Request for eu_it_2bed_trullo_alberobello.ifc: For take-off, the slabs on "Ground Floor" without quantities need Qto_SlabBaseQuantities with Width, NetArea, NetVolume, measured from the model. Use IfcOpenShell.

First a look at what the model holds.

```python
import ifcopenshell
import ifcopenshell.util.element
import ifcopenshell.util.unit

model = ifcopenshell.open("eu_it_2bed_trullo_alberobello.ifc")
print(model.schema)
for unit_type in ("LENGTHUNIT", "AREAUNIT", "VOLUMEUNIT"):
    print(unit_type, ifcopenshell.util.unit.calculate_unit_scale(model, unit_type))
storey = next(s for s in model.by_type("IfcBuildingStorey") if s.Name == "Ground Floor")
slabs = [e for e in ifcopenshell.util.element.get_decomposition(storey) if e.is_a("IfcSlab")]
for e in sorted(slabs, key=lambda e: e.id()):
    print(e.id(), e.is_a(), e.Name, list(ifcopenshell.util.element.get_psets(e, qtos_only=True)), sep=" | ")
```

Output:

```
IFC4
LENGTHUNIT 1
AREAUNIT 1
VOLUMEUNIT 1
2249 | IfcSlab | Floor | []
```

```python
import ifcopenshell
import ifcopenshell.api.pset
import ifcopenshell.geom
import ifcopenshell.util.element
import ifcopenshell.util.shape
import ifcopenshell.util.unit

model = ifcopenshell.open("eu_it_2bed_trullo_alberobello.ifc")
unit_scale = ifcopenshell.util.unit.calculate_unit_scale(model)
area_scale = ifcopenshell.util.unit.calculate_unit_scale(model, "AREAUNIT")
volume_scale = ifcopenshell.util.unit.calculate_unit_scale(model, "VOLUMEUNIT")
settings = ifcopenshell.geom.settings()

storey = next(s for s in model.by_type("IfcBuildingStorey") if s.Name == "Ground Floor")
slabs = [e for e in ifcopenshell.util.element.get_decomposition(storey) if e.is_a("IfcSlab")]

for e in sorted(slabs, key=lambda e: e.id()):
    if ifcopenshell.util.element.get_psets(e, qtos_only=True, should_inherit=False):
        continue
    # Geometry comes back in metres, in the element's own axes.
    shape = ifcopenshell.geom.create_shape(settings, e)
    values = {
        "Width": ifcopenshell.util.shape.get_z(shape.geometry) / unit_scale,
        "NetArea": ifcopenshell.util.shape.get_footprint_area(shape.geometry) / area_scale,
        "NetVolume": ifcopenshell.util.shape.get_volume(shape.geometry) / volume_scale,
    }
    qto = ifcopenshell.api.pset.add_qto(model, product=e, name="Qto_SlabBaseQuantities")
    ifcopenshell.api.pset.edit_qto(model, qto=qto, properties=values)
    print(e.id(), {k: round(v, 3) for k, v in values.items()})

model.write("eu_it_2bed_trullo_alberobello-out.ifc")
```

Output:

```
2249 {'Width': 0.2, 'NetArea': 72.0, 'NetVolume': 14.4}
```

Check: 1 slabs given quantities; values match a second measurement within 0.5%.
